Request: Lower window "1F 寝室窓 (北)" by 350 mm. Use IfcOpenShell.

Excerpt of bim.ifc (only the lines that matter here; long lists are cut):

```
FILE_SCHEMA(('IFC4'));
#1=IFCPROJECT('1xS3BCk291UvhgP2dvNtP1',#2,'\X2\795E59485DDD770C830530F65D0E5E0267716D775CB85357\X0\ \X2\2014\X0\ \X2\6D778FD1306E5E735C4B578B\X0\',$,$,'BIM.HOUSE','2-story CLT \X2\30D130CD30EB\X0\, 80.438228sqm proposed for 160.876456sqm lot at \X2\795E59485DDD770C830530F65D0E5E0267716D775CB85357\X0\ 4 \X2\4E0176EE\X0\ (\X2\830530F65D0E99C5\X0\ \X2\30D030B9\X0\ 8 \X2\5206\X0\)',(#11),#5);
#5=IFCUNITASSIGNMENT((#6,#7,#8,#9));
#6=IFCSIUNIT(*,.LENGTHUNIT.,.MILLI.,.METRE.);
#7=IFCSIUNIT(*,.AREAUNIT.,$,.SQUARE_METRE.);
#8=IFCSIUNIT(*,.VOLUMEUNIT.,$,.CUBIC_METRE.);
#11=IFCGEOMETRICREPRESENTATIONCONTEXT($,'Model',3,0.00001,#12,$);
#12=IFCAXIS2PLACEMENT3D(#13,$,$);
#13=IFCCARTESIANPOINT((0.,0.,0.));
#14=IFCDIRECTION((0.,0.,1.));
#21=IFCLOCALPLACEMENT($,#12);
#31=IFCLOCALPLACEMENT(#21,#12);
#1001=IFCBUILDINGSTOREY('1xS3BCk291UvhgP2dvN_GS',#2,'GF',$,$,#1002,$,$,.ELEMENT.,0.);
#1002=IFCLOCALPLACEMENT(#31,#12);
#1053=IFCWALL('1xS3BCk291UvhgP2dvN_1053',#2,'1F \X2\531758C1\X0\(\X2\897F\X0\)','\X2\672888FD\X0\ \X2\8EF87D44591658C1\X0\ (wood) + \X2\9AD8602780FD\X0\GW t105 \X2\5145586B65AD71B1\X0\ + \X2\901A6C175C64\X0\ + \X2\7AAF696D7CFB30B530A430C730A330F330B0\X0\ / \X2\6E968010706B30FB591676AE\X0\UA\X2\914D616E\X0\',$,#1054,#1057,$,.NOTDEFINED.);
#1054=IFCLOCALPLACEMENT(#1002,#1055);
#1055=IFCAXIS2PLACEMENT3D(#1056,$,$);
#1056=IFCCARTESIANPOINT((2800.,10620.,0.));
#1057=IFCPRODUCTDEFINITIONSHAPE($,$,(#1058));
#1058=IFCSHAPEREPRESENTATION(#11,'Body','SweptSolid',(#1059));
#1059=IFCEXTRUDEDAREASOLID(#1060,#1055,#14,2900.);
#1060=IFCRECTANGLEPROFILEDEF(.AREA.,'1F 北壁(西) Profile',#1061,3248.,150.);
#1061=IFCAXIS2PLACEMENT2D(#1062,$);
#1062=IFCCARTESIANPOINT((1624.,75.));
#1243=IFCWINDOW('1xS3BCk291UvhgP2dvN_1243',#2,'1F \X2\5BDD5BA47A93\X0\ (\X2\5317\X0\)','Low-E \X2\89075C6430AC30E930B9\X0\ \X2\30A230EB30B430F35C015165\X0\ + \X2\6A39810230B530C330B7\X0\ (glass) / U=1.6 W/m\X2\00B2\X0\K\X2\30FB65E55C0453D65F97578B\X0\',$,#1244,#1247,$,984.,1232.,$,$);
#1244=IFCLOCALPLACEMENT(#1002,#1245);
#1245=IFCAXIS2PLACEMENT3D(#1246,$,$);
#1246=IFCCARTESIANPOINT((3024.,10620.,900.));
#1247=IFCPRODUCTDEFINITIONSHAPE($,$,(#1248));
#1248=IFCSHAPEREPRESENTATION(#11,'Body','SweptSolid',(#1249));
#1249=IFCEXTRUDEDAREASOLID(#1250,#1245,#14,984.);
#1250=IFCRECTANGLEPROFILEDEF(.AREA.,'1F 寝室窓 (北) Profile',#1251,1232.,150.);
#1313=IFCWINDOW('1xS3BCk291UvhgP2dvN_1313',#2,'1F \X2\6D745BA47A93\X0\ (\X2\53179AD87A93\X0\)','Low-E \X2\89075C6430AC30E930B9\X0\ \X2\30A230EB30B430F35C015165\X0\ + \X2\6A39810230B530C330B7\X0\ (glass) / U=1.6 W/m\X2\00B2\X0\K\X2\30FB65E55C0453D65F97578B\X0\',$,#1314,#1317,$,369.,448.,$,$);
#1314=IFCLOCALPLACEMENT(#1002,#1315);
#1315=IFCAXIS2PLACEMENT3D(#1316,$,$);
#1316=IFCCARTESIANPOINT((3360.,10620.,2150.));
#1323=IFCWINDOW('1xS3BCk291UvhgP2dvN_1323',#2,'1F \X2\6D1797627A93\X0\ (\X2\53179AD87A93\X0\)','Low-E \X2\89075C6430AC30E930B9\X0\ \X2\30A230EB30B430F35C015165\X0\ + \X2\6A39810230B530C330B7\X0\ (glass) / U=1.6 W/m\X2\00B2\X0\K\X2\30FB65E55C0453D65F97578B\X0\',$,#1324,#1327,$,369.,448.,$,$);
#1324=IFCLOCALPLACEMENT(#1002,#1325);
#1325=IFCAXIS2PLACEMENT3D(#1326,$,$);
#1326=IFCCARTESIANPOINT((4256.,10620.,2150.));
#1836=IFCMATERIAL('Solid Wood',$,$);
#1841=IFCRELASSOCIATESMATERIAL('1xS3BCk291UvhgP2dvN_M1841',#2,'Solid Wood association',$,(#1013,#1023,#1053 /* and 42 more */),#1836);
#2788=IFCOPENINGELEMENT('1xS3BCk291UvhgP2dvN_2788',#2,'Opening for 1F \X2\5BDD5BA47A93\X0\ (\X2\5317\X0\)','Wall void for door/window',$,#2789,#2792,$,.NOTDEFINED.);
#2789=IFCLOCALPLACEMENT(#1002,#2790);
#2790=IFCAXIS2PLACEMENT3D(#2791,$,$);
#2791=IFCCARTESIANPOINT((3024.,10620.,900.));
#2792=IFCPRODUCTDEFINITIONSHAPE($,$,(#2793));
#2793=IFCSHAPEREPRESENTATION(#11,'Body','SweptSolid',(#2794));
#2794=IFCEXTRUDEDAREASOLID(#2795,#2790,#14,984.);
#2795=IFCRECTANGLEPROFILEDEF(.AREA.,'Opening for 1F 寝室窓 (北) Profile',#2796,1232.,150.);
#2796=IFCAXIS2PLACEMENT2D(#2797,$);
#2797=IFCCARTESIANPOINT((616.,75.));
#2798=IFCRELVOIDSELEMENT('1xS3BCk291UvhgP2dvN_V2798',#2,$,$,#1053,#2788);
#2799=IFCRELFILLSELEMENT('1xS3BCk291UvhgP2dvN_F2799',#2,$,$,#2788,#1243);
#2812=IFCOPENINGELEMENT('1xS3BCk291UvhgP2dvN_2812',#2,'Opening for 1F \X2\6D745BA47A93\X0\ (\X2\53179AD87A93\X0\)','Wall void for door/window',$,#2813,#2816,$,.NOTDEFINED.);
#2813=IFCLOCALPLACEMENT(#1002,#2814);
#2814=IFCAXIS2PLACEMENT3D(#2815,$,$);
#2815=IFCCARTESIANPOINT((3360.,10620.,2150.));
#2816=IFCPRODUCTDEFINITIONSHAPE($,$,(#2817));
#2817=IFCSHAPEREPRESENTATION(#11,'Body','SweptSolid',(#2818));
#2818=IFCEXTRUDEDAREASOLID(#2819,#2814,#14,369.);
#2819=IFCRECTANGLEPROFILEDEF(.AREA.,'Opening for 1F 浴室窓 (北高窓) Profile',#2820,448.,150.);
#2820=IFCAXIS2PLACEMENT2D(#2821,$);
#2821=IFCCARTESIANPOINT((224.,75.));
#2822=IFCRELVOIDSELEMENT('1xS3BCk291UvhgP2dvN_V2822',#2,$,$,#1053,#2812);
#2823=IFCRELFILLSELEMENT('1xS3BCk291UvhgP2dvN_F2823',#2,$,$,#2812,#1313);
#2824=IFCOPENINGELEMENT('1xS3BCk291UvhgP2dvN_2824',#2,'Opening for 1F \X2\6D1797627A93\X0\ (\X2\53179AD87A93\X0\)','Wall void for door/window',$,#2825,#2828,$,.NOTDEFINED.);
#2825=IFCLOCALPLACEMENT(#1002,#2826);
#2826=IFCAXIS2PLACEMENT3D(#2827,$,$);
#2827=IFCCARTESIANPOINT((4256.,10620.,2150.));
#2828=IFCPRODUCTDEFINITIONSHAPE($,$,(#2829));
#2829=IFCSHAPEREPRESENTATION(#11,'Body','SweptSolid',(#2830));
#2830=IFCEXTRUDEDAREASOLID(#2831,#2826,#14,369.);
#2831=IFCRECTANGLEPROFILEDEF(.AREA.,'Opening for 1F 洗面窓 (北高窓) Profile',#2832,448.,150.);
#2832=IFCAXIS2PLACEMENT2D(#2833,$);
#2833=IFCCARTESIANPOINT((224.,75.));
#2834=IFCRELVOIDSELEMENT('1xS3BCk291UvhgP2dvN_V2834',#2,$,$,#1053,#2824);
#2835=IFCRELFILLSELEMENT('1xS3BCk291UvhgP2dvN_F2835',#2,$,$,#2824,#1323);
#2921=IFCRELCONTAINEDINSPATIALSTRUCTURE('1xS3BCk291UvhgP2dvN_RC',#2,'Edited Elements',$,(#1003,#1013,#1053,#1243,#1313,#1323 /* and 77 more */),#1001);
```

```python
import numpy as np
import ifcopenshell
import ifcopenshell.api.geometry
import ifcopenshell.util.placement
import ifcopenshell.util.unit

model = ifcopenshell.open("bim.ifc")
unit_scale = ifcopenshell.util.unit.calculate_unit_scale(model)

window = model.by_guid("1xS3BCk291UvhgP2dvN_1243")
opening = window.FillsVoids[0].RelatingOpeningElement
dz = -350.0

shift = np.array([0.0, 0.0, dz])
# The window is not placed relative to its opening, so move both.
for product in (opening, window):
    matrix = ifcopenshell.util.placement.get_local_placement(product.ObjectPlacement)
    matrix[:3, 3] += shift
    ifcopenshell.api.geometry.edit_object_placement(model, product=product, matrix=matrix, is_si=False)

print(f"moved by {dz * unit_scale:+.3f} m")

model.write("bim_v2.ifc")
```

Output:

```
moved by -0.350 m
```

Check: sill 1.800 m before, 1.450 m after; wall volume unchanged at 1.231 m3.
